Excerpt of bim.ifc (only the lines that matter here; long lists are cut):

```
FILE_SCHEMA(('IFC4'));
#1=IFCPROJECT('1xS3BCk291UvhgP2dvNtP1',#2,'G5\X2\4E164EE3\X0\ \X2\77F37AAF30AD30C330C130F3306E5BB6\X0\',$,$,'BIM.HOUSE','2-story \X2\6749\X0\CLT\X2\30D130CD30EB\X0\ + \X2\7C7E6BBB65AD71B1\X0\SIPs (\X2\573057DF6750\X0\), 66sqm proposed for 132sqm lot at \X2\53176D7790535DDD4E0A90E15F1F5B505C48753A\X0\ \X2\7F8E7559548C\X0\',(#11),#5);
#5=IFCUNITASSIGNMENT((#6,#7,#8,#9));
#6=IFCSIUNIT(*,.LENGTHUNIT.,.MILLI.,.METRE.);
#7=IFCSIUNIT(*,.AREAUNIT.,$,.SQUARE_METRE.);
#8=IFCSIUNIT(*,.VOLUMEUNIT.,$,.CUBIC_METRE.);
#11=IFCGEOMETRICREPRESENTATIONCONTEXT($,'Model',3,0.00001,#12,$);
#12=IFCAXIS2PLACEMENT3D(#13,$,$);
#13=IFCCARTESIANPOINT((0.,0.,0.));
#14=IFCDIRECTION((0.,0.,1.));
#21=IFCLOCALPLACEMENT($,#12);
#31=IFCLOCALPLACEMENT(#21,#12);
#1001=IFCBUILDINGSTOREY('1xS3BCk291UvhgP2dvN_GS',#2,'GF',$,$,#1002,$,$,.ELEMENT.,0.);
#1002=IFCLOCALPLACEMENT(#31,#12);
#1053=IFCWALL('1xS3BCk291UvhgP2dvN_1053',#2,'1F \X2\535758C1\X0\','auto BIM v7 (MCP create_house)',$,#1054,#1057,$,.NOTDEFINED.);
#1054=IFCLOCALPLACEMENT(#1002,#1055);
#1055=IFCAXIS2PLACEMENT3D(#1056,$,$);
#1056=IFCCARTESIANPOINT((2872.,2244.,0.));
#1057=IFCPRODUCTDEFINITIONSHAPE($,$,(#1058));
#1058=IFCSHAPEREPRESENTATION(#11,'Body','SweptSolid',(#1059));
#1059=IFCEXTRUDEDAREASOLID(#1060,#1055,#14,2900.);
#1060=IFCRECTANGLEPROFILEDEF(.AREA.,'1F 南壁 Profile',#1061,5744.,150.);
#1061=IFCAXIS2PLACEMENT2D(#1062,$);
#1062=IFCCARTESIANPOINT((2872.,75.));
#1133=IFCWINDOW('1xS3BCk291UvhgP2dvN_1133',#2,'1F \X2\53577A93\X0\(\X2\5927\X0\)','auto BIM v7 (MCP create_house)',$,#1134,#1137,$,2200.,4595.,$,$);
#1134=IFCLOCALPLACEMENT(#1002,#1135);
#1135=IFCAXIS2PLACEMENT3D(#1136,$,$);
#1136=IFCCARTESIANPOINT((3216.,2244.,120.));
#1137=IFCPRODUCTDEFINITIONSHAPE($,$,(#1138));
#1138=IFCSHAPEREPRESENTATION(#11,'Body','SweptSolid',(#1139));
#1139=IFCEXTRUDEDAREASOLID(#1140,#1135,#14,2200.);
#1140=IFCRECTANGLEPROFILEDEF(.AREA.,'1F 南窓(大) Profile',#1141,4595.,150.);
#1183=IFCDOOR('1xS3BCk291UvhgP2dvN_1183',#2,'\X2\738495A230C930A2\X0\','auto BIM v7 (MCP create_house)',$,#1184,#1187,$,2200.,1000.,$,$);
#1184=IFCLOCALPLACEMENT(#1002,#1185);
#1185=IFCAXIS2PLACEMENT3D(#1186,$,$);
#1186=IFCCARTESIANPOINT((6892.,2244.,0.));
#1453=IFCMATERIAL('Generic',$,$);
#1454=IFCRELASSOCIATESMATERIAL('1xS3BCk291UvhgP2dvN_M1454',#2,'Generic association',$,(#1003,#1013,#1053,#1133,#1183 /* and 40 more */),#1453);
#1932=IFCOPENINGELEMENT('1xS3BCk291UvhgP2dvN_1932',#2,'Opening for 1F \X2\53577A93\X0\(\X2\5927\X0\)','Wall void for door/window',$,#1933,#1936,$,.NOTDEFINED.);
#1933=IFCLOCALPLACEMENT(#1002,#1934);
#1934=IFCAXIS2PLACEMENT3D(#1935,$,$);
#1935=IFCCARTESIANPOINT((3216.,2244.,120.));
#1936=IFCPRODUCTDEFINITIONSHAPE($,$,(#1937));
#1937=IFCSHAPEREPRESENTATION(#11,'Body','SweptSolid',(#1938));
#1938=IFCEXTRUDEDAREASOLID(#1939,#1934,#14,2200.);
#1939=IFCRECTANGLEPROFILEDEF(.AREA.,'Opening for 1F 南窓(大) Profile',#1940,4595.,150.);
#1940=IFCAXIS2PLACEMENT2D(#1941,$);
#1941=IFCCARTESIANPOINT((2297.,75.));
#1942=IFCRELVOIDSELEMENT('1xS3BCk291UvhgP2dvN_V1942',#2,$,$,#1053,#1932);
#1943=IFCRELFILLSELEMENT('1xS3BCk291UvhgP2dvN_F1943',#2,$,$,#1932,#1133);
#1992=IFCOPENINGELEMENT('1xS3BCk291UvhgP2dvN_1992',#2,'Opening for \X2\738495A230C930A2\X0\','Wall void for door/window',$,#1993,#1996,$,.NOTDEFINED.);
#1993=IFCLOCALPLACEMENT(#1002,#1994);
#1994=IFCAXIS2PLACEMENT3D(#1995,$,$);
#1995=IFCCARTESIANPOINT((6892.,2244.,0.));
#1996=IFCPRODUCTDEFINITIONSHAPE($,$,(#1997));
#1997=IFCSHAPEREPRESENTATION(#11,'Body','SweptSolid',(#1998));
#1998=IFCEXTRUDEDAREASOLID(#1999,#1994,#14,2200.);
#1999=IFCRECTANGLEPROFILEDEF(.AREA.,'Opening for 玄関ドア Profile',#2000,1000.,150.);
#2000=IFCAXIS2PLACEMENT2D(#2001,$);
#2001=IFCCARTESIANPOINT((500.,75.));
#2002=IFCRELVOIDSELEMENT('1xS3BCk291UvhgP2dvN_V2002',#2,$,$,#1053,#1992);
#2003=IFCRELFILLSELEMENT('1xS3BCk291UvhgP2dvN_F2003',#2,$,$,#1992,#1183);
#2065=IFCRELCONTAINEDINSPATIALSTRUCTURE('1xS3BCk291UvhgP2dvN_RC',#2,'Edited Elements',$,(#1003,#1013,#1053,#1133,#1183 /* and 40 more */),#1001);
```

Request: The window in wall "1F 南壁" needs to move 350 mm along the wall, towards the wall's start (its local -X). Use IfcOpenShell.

```python
import ifcopenshell
import ifcopenshell.api.geometry
import ifcopenshell.util.placement

model = ifcopenshell.open("bim.ifc")

window = model.by_id(1133)
opening = window.FillsVoids[0].RelatingOpeningElement
wall = opening.VoidsElements[0].RelatingBuildingElement

wall_matrix = ifcopenshell.util.placement.get_local_placement(wall.ObjectPlacement)
shift = wall_matrix[:3, 0] * -350.0
before = ifcopenshell.util.placement.get_local_placement(window.ObjectPlacement)[:3, 3].copy()

# The window is not placed relative to its opening, so move both.
for product in (opening, window):
    matrix = ifcopenshell.util.placement.get_local_placement(product.ObjectPlacement)
    matrix[:3, 3] += shift
    ifcopenshell.api.geometry.edit_object_placement(model, product=product, matrix=matrix, is_si=False)

after = ifcopenshell.util.placement.get_local_placement(window.ObjectPlacement)[:3, 3]
print("window moved by", (after - before).round(3) + 0.0)

model.write("bim_v2.ifc")
```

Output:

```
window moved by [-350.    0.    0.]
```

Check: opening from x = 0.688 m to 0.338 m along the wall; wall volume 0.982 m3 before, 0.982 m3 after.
